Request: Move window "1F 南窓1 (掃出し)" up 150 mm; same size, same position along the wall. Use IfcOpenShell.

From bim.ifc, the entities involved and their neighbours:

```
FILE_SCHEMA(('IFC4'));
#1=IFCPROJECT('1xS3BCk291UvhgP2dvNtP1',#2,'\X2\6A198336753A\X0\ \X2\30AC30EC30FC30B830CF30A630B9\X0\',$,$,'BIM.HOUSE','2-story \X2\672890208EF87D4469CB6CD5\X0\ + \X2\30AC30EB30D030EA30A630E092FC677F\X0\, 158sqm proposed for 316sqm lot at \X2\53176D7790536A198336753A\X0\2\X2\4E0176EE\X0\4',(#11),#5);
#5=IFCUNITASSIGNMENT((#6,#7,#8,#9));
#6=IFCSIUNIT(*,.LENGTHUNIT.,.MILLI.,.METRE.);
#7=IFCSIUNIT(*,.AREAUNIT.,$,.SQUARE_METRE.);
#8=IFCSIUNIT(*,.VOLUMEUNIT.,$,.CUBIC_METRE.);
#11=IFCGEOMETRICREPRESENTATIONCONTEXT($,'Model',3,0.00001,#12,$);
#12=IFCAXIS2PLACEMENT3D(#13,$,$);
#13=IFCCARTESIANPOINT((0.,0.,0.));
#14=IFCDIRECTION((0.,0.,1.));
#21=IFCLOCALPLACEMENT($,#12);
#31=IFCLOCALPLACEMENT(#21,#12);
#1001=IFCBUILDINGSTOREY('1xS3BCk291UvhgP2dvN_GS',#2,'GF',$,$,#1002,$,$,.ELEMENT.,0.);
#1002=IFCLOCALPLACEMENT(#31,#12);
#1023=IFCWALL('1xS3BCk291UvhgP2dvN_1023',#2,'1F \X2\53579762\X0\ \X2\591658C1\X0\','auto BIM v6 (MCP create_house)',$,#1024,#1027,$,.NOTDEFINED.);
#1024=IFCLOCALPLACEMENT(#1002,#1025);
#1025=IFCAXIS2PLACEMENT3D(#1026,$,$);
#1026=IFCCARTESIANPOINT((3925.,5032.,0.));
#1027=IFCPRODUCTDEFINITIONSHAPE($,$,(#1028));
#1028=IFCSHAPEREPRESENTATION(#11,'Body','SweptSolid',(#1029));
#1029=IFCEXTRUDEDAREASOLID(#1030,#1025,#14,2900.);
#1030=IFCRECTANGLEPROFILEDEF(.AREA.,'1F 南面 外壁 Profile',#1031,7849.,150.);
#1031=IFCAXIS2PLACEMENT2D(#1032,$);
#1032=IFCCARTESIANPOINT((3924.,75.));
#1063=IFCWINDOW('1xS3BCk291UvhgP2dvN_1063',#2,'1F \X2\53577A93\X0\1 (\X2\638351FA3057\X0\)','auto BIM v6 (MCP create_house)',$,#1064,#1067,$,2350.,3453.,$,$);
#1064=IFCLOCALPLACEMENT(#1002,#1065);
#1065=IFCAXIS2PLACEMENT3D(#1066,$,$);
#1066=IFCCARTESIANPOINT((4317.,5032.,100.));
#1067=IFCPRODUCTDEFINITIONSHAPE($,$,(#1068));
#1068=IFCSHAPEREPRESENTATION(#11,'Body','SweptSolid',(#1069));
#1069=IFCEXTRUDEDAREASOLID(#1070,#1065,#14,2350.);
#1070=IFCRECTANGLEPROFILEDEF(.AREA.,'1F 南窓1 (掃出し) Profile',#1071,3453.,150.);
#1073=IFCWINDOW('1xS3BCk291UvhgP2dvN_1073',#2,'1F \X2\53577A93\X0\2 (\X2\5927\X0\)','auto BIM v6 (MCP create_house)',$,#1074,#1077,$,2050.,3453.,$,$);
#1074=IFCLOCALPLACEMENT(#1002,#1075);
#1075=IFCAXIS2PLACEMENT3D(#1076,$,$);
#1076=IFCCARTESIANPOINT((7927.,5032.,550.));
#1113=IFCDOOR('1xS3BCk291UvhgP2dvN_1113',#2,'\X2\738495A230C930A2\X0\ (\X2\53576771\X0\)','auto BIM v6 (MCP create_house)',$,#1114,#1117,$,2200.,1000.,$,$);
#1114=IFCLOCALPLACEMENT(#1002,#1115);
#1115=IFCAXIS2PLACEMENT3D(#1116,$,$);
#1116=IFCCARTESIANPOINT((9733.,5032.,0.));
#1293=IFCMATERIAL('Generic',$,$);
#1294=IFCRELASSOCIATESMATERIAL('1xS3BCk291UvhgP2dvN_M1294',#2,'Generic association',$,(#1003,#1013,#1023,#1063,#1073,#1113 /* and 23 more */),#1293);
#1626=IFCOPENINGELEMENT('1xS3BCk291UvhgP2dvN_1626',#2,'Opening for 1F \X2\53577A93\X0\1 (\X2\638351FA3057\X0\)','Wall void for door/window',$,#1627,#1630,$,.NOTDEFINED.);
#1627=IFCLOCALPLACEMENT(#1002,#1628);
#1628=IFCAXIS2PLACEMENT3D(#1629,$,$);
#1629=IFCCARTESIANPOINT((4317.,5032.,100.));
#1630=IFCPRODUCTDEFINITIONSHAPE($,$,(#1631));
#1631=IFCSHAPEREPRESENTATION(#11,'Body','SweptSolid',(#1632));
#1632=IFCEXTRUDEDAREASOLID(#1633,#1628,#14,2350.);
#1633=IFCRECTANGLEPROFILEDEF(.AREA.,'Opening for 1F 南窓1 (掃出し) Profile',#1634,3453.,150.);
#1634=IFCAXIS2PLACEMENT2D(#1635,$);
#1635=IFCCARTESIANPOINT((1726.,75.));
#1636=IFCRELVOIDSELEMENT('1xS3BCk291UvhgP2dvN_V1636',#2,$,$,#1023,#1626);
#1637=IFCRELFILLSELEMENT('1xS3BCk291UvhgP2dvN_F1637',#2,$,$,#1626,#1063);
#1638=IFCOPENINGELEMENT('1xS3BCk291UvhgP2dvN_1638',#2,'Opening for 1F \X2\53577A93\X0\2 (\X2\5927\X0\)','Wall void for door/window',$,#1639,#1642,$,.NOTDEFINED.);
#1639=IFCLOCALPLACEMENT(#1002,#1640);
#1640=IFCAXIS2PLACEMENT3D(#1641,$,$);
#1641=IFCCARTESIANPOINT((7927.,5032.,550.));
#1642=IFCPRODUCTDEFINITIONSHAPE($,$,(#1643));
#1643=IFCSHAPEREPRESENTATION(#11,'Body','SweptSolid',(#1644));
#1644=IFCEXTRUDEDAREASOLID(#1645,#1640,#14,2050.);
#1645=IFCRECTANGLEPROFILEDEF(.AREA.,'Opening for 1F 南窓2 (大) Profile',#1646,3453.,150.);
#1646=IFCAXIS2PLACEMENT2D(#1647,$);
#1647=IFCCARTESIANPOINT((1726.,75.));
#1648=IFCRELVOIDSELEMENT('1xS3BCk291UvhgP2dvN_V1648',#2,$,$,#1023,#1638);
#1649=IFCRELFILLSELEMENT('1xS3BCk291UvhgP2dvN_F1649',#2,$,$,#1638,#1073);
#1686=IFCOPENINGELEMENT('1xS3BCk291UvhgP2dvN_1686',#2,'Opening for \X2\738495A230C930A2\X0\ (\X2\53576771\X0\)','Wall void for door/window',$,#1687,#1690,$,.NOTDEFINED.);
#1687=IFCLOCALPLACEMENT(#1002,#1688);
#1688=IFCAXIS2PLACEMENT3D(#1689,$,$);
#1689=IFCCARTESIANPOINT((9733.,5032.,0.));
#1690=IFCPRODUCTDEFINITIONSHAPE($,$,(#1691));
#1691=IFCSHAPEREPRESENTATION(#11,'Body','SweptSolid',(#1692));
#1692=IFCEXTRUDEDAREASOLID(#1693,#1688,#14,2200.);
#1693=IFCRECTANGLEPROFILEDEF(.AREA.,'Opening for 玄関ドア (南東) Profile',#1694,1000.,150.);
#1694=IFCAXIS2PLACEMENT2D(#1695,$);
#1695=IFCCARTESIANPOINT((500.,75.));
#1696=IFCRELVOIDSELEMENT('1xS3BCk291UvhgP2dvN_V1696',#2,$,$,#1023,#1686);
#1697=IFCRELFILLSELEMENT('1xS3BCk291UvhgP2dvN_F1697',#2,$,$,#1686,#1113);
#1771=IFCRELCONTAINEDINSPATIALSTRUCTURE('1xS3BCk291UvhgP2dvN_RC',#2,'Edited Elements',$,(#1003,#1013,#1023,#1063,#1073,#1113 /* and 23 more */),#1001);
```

```python
import numpy as np
import ifcopenshell
import ifcopenshell.api.geometry
import ifcopenshell.util.placement
import ifcopenshell.util.unit

model = ifcopenshell.open("bim.ifc")
unit_scale = ifcopenshell.util.unit.calculate_unit_scale(model)

window = model.by_guid("1xS3BCk291UvhgP2dvN_1063")
opening = window.FillsVoids[0].RelatingOpeningElement
dz = 0.15 / unit_scale

shift = np.array([0.0, 0.0, dz])
# The window is not placed relative to its opening, so move both.
for product in (opening, window):
    matrix = ifcopenshell.util.placement.get_local_placement(product.ObjectPlacement)
    matrix[:3, 3] += shift
    ifcopenshell.api.geometry.edit_object_placement(model, product=product, matrix=matrix, is_si=False)

print(f"moved by {dz * unit_scale:+.3f} m")

model.write("bim_v2.ifc")
```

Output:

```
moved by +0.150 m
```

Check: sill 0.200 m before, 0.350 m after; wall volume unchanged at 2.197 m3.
